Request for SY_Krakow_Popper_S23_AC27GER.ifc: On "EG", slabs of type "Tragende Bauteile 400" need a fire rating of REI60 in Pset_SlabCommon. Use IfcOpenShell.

First a look at what the model holds.

```python
import ifcopenshell
import ifcopenshell.util.element

model = ifcopenshell.open("SY_Krakow_Popper_S23_AC27GER.ifc")
print(model.schema)
storey = next(s for s in model.by_type("IfcBuildingStorey") if s.Name == "EG")
slabs = [e for e in ifcopenshell.util.element.get_decomposition(storey) if e.is_a("IfcSlab")]
seen = {}
for e in slabs:
    element_type = ifcopenshell.util.element.get_type(e)
    key = (element_type.Name if element_type != e and element_type else None, ifcopenshell.util.element.get_pset(e, "Pset_SlabCommon", "FireRating"))
    seen[key] = seen.get(key, 0) + 1
for (name, value), count in sorted(seen.items(), key=str):
    print(count, "x", name, "|", value)
```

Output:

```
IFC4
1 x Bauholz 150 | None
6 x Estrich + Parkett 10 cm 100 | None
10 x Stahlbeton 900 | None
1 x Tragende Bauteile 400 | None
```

```python
import ifcopenshell
import ifcopenshell.api.pset
import ifcopenshell.util.element

model = ifcopenshell.open("SY_Krakow_Popper_S23_AC27GER.ifc")

storey = next(s for s in model.by_type("IfcBuildingStorey") if s.Name == "EG")
slabs = [e for e in ifcopenshell.util.element.get_decomposition(storey) if e.is_a("IfcSlab")]

count = 0
for e in slabs:
    element_type = ifcopenshell.util.element.get_type(e)
    if element_type in (None, e) or element_type.Name != "Tragende Bauteile 400":
        continue
    # add_pset returns the element's existing set when there is one.
    pset = ifcopenshell.api.pset.add_pset(model, product=e, name="Pset_SlabCommon")
    ifcopenshell.api.pset.edit_pset(model, pset=pset, properties={"FireRating": "REI60"})
    count += 1

print(count, "slabs updated")

model.write("SY_Krakow_Popper_S23_AC27GER_edited.ifc")
```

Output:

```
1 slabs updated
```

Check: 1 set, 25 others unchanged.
